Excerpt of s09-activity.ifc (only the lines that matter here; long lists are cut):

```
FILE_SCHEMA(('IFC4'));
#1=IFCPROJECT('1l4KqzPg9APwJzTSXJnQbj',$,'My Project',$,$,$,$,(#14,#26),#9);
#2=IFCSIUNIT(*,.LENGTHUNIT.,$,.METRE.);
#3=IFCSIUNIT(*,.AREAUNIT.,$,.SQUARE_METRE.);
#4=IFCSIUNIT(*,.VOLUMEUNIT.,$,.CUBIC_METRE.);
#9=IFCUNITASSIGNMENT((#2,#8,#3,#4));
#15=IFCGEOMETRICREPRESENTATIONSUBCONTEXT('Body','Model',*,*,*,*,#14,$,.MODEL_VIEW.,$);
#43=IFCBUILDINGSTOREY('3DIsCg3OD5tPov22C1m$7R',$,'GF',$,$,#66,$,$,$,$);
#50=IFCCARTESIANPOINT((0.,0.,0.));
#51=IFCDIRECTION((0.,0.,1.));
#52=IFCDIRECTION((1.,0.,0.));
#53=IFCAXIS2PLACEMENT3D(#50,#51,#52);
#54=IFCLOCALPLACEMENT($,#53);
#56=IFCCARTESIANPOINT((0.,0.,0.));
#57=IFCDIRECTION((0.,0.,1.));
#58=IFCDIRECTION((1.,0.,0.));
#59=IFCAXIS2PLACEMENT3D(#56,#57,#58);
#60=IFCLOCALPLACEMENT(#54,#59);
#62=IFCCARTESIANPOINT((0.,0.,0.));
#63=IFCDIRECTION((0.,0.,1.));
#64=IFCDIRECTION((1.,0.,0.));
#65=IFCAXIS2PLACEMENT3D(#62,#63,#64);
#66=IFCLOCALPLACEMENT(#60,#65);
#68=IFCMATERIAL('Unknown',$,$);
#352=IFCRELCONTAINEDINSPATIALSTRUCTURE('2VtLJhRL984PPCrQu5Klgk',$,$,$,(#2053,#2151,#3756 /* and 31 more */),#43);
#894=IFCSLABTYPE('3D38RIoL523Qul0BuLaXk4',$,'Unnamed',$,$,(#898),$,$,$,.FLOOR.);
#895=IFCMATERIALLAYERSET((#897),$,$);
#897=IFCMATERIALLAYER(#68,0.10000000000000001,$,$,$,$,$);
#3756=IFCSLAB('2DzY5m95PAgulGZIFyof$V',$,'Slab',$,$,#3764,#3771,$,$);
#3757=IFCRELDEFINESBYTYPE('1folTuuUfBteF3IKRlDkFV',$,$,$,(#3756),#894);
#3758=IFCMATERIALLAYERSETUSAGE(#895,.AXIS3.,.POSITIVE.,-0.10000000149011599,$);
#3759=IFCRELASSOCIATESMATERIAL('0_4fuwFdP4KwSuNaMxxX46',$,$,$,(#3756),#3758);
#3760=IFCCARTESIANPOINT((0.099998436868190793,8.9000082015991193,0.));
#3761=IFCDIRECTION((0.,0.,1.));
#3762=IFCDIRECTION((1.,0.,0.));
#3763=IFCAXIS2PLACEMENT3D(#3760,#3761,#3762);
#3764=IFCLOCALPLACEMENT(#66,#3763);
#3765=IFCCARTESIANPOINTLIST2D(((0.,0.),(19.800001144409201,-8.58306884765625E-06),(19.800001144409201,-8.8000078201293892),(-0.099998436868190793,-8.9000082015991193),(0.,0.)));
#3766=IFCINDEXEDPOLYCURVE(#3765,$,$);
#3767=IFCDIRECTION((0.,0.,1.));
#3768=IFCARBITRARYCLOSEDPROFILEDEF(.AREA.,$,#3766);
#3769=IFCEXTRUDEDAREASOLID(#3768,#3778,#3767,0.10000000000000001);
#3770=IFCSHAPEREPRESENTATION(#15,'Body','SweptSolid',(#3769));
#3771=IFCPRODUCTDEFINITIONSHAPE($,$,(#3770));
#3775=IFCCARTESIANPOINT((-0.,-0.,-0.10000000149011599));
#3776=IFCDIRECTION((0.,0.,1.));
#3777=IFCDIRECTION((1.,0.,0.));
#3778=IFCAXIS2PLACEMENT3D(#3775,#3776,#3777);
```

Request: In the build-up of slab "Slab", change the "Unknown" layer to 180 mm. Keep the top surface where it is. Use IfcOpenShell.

```python
import ifcopenshell
import ifcopenshell.util.element
import ifcopenshell.util.representation

model = ifcopenshell.open("s09-activity.ifc")

layer_set = model.by_id(895)
layer = next(l for l in layer_set.MaterialLayers if l.Material and l.Material.Name == "Unknown")
change = 0.18 - layer.LayerThickness
layer.LayerThickness += change

# Geometry does not follow the layer set by itself.
slabs = [e for e in ifcopenshell.util.element.get_elements_by_material(model, layer_set) if e.is_a("IfcSlab")]
for slab in sorted(slabs, key=lambda e: e.id()):
    body = ifcopenshell.util.representation.get_representation(slab, "Model", "Body")
    solid = body.Items[0]
    old_depth = solid.Depth
    solid.Depth += change
    # Extruded upwards: lower the start of the extrusion so the top stays.
    x, y, z = solid.Position.Location.Coordinates
    solid.Position.Location = model.createIfcCartesianPoint((x, y, z - change))
    print(slab.id(), f"{old_depth:g} -> {solid.Depth:g}")

# The layers are counted up from the underside, which has moved.
for usage in {ifcopenshell.util.element.get_material(slab) for slab in slabs}:
    usage.OffsetFromReferenceLine -= change

model.write("s09-activity-out.ifc")
```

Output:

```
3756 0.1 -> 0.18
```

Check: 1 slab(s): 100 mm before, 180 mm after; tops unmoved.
